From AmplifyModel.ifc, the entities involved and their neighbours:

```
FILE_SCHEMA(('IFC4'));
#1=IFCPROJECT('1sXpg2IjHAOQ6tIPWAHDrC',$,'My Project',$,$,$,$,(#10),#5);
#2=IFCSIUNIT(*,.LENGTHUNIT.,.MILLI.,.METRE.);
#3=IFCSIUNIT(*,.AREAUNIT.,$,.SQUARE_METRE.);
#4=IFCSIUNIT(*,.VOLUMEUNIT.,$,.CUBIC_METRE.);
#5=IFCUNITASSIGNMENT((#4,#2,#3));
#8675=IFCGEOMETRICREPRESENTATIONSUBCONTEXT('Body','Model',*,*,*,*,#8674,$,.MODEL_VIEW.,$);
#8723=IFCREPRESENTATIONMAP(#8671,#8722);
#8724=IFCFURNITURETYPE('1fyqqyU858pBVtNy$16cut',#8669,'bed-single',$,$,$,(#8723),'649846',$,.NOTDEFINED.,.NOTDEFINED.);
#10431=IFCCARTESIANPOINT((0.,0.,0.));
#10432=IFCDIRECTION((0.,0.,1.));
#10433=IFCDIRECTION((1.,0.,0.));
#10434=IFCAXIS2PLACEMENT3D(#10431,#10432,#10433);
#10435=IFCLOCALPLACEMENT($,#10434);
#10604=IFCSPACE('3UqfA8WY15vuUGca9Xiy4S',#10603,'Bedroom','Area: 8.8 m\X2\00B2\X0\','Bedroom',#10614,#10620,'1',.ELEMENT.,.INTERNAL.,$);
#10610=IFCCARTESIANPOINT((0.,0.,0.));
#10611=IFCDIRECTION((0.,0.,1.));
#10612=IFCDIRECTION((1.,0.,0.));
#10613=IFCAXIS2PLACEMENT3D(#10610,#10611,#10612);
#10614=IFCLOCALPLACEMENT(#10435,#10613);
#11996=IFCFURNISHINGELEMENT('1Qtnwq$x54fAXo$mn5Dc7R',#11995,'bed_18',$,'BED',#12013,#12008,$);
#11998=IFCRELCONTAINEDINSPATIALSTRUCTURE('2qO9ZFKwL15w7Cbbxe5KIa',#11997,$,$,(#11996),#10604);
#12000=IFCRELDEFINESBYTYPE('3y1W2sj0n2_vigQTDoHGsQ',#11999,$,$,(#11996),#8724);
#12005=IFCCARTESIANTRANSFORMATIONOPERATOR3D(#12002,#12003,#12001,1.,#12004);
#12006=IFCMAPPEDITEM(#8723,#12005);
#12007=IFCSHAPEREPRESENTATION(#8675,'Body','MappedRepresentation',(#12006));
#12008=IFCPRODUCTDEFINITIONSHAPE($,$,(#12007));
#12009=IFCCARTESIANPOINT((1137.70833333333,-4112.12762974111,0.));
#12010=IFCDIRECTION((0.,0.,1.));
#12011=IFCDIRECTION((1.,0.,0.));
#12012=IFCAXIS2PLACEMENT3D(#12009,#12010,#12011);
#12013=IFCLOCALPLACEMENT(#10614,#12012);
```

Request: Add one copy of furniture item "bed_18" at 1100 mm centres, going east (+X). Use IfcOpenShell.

```python
import numpy as np
import ifcopenshell
import ifcopenshell.api.geometry
import ifcopenshell.api.root
import ifcopenshell.util.element
import ifcopenshell.util.placement

model = ifcopenshell.open("AmplifyModel.ifc")

source = model.by_guid("1Qtnwq$x54fAXo$mn5Dc7R")
base = ifcopenshell.util.placement.get_local_placement(source.ObjectPlacement)
step = np.array([1.0, 0.0, 0.0]) * 1100.0

for i in range(1, 2):
    copy = ifcopenshell.api.root.copy_class(model, product=source)
    copy.Representation = ifcopenshell.util.element.copy_deep(
        model, source.Representation, exclude=["IfcGeometricRepresentationContext", "IfcRepresentationMap"]
    )
    matrix = base.copy()
    matrix[:3, 3] += i * step
    print("added at", matrix[:3, 3].round(3) + 0.0)
    ifcopenshell.api.geometry.edit_object_placement(model, product=copy, matrix=matrix, is_si=False)

model.write("AmplifyModel_edited.ifc")
```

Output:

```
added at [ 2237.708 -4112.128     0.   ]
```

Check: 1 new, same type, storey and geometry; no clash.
